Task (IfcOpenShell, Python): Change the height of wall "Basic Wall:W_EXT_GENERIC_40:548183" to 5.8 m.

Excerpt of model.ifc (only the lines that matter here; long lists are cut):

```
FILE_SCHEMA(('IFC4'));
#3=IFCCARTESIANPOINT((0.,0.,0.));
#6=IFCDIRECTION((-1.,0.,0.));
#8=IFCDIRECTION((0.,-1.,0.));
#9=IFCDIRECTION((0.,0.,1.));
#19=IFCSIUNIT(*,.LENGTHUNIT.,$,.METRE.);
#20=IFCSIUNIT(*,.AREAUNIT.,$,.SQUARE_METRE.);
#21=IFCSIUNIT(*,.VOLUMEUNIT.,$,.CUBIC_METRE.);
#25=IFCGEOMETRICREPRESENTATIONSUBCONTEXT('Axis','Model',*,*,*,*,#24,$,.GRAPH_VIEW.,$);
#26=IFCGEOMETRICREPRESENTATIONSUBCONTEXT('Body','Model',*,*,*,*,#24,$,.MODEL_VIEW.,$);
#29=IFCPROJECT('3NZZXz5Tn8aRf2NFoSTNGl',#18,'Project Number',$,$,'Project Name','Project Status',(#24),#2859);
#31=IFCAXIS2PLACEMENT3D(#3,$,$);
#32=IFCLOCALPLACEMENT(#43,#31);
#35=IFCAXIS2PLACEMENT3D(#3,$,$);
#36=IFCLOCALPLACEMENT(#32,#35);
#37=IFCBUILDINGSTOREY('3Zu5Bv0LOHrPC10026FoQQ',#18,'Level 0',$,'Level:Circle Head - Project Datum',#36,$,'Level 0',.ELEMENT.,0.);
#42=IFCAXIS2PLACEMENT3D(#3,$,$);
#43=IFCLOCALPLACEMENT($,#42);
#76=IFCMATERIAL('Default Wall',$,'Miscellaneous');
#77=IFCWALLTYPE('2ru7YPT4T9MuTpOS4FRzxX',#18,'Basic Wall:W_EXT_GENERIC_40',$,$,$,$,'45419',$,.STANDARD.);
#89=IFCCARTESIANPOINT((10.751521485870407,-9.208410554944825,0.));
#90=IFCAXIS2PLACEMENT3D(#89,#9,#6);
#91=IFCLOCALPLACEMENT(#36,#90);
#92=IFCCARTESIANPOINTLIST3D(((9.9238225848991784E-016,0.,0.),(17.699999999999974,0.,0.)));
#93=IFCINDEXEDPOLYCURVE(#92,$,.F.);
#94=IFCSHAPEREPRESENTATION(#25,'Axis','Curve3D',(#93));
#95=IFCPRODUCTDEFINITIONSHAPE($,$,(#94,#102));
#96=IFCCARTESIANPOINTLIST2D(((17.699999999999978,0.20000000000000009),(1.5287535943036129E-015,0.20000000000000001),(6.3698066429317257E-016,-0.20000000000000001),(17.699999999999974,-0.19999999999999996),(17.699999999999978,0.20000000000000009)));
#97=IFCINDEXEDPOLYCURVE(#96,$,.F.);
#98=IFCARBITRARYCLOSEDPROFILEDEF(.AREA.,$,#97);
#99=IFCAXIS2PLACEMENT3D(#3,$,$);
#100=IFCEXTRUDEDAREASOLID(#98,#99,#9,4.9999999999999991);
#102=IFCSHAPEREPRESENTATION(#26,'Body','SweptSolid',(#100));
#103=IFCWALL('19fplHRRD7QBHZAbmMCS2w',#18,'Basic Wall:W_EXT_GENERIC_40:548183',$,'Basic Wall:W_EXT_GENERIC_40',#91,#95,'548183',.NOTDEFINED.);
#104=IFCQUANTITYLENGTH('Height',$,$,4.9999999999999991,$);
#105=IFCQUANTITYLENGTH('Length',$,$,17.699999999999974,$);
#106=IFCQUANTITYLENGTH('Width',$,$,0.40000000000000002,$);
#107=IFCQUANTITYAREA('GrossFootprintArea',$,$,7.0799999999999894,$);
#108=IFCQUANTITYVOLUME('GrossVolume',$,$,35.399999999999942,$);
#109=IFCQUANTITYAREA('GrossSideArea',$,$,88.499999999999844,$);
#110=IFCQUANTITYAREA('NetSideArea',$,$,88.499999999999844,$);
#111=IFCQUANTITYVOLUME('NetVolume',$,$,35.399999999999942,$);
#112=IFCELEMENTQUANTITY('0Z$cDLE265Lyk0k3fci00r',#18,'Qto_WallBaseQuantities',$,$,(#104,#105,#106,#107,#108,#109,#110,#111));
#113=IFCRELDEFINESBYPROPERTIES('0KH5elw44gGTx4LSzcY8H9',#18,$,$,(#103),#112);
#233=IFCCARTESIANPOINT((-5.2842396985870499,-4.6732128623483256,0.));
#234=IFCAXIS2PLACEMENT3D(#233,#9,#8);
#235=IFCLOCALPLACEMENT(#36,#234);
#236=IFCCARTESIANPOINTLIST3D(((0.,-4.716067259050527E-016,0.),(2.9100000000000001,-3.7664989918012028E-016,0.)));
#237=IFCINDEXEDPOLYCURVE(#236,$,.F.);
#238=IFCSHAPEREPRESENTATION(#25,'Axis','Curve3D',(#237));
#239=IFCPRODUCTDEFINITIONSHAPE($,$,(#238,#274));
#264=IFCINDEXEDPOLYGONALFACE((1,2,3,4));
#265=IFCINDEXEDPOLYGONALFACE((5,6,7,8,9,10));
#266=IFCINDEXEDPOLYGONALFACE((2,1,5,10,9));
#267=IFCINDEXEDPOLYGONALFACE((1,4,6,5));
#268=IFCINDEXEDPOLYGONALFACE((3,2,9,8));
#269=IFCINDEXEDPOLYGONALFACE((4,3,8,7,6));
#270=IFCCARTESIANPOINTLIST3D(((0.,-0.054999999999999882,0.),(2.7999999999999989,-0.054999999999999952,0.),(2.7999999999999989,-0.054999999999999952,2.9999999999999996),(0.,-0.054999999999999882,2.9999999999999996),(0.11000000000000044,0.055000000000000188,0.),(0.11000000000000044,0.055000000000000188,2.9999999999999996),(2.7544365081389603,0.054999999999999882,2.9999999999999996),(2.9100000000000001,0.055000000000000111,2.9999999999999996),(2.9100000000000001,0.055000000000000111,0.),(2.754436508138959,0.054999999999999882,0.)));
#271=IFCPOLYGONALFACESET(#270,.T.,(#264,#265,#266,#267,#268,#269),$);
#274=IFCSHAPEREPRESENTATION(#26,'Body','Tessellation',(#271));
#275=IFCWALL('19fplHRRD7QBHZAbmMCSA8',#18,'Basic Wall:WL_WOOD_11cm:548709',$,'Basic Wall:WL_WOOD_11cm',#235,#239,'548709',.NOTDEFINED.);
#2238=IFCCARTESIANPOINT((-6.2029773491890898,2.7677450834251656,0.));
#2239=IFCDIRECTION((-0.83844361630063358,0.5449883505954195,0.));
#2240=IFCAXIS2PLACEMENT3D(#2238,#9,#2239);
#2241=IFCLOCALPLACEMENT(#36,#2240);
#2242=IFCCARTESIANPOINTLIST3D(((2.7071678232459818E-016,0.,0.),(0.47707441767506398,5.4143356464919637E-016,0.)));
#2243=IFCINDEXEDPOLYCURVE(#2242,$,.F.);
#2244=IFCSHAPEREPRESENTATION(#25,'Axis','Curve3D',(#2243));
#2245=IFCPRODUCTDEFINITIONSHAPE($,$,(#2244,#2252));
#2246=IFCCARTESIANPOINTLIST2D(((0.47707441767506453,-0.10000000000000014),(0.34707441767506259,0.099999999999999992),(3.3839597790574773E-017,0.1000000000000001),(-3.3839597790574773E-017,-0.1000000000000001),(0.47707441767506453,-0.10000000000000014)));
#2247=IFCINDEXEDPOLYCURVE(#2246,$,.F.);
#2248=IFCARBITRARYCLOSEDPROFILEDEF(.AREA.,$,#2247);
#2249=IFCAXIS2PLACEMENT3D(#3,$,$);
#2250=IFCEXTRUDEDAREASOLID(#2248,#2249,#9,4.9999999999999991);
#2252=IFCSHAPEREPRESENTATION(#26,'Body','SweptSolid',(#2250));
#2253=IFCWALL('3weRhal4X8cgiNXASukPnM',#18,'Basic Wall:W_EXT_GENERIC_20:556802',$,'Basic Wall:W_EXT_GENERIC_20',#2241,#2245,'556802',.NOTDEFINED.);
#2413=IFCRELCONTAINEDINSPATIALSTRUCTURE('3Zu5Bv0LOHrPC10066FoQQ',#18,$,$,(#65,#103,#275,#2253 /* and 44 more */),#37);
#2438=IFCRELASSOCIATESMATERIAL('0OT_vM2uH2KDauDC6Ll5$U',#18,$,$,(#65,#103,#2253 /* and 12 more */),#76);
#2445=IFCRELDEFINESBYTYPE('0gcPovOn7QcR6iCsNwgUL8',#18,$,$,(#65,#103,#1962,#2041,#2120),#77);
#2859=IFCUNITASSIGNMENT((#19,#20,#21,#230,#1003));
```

```python
import ifcopenshell
import ifcopenshell.api.pset
import ifcopenshell.geom
import ifcopenshell.util.element
import ifcopenshell.util.representation
import ifcopenshell.util.shape
import ifcopenshell.util.unit

model = ifcopenshell.open("model.ifc")
unit_scale = ifcopenshell.util.unit.calculate_unit_scale(model)
area_scale = ifcopenshell.util.unit.calculate_unit_scale(model, "AREAUNIT")
volume_scale = ifcopenshell.util.unit.calculate_unit_scale(model, "VOLUMEUNIT")
settings = ifcopenshell.geom.settings()


def volume(element):
    """Net volume in cubic metres, openings subtracted."""
    shape = ifcopenshell.geom.create_shape(settings, element)
    return ifcopenshell.util.shape.get_volume(shape.geometry)


wall = model.by_guid("19fplHRRD7QBHZAbmMCS2w")
before = volume(wall)

body = ifcopenshell.util.representation.get_representation(wall, "Model", "Body")
solid = body.Items[0]
old_height = solid.Depth
solid.Depth = 5.8 / unit_scale
after = volume(wall)
thickness = 0.4  # wall thickness in metres

# Update the stored height, areas and volumes.
qto = model.by_id(ifcopenshell.util.element.get_pset(wall, "Qto_WallBaseQuantities", should_inherit=False)["id"])
ifcopenshell.api.pset.edit_qto(model, qto=qto, properties={
    "Height": solid.Depth,
    "GrossVolume": ifcopenshell.util.element.get_pset(wall, "Qto_WallBaseQuantities", "GrossVolume") * solid.Depth / old_height,
    "GrossSideArea": ifcopenshell.util.element.get_pset(wall, "Qto_WallBaseQuantities", "GrossSideArea") * solid.Depth / old_height,
    "NetSideArea": after / thickness / area_scale,
    "NetVolume": after / volume_scale,
})

print(f"height {old_height:g} -> {solid.Depth:g}, volume {before:.3f} -> {after:.3f} m3")

model.write("model_updated.ifc")
```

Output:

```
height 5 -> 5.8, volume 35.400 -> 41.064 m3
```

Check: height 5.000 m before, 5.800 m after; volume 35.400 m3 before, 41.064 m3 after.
